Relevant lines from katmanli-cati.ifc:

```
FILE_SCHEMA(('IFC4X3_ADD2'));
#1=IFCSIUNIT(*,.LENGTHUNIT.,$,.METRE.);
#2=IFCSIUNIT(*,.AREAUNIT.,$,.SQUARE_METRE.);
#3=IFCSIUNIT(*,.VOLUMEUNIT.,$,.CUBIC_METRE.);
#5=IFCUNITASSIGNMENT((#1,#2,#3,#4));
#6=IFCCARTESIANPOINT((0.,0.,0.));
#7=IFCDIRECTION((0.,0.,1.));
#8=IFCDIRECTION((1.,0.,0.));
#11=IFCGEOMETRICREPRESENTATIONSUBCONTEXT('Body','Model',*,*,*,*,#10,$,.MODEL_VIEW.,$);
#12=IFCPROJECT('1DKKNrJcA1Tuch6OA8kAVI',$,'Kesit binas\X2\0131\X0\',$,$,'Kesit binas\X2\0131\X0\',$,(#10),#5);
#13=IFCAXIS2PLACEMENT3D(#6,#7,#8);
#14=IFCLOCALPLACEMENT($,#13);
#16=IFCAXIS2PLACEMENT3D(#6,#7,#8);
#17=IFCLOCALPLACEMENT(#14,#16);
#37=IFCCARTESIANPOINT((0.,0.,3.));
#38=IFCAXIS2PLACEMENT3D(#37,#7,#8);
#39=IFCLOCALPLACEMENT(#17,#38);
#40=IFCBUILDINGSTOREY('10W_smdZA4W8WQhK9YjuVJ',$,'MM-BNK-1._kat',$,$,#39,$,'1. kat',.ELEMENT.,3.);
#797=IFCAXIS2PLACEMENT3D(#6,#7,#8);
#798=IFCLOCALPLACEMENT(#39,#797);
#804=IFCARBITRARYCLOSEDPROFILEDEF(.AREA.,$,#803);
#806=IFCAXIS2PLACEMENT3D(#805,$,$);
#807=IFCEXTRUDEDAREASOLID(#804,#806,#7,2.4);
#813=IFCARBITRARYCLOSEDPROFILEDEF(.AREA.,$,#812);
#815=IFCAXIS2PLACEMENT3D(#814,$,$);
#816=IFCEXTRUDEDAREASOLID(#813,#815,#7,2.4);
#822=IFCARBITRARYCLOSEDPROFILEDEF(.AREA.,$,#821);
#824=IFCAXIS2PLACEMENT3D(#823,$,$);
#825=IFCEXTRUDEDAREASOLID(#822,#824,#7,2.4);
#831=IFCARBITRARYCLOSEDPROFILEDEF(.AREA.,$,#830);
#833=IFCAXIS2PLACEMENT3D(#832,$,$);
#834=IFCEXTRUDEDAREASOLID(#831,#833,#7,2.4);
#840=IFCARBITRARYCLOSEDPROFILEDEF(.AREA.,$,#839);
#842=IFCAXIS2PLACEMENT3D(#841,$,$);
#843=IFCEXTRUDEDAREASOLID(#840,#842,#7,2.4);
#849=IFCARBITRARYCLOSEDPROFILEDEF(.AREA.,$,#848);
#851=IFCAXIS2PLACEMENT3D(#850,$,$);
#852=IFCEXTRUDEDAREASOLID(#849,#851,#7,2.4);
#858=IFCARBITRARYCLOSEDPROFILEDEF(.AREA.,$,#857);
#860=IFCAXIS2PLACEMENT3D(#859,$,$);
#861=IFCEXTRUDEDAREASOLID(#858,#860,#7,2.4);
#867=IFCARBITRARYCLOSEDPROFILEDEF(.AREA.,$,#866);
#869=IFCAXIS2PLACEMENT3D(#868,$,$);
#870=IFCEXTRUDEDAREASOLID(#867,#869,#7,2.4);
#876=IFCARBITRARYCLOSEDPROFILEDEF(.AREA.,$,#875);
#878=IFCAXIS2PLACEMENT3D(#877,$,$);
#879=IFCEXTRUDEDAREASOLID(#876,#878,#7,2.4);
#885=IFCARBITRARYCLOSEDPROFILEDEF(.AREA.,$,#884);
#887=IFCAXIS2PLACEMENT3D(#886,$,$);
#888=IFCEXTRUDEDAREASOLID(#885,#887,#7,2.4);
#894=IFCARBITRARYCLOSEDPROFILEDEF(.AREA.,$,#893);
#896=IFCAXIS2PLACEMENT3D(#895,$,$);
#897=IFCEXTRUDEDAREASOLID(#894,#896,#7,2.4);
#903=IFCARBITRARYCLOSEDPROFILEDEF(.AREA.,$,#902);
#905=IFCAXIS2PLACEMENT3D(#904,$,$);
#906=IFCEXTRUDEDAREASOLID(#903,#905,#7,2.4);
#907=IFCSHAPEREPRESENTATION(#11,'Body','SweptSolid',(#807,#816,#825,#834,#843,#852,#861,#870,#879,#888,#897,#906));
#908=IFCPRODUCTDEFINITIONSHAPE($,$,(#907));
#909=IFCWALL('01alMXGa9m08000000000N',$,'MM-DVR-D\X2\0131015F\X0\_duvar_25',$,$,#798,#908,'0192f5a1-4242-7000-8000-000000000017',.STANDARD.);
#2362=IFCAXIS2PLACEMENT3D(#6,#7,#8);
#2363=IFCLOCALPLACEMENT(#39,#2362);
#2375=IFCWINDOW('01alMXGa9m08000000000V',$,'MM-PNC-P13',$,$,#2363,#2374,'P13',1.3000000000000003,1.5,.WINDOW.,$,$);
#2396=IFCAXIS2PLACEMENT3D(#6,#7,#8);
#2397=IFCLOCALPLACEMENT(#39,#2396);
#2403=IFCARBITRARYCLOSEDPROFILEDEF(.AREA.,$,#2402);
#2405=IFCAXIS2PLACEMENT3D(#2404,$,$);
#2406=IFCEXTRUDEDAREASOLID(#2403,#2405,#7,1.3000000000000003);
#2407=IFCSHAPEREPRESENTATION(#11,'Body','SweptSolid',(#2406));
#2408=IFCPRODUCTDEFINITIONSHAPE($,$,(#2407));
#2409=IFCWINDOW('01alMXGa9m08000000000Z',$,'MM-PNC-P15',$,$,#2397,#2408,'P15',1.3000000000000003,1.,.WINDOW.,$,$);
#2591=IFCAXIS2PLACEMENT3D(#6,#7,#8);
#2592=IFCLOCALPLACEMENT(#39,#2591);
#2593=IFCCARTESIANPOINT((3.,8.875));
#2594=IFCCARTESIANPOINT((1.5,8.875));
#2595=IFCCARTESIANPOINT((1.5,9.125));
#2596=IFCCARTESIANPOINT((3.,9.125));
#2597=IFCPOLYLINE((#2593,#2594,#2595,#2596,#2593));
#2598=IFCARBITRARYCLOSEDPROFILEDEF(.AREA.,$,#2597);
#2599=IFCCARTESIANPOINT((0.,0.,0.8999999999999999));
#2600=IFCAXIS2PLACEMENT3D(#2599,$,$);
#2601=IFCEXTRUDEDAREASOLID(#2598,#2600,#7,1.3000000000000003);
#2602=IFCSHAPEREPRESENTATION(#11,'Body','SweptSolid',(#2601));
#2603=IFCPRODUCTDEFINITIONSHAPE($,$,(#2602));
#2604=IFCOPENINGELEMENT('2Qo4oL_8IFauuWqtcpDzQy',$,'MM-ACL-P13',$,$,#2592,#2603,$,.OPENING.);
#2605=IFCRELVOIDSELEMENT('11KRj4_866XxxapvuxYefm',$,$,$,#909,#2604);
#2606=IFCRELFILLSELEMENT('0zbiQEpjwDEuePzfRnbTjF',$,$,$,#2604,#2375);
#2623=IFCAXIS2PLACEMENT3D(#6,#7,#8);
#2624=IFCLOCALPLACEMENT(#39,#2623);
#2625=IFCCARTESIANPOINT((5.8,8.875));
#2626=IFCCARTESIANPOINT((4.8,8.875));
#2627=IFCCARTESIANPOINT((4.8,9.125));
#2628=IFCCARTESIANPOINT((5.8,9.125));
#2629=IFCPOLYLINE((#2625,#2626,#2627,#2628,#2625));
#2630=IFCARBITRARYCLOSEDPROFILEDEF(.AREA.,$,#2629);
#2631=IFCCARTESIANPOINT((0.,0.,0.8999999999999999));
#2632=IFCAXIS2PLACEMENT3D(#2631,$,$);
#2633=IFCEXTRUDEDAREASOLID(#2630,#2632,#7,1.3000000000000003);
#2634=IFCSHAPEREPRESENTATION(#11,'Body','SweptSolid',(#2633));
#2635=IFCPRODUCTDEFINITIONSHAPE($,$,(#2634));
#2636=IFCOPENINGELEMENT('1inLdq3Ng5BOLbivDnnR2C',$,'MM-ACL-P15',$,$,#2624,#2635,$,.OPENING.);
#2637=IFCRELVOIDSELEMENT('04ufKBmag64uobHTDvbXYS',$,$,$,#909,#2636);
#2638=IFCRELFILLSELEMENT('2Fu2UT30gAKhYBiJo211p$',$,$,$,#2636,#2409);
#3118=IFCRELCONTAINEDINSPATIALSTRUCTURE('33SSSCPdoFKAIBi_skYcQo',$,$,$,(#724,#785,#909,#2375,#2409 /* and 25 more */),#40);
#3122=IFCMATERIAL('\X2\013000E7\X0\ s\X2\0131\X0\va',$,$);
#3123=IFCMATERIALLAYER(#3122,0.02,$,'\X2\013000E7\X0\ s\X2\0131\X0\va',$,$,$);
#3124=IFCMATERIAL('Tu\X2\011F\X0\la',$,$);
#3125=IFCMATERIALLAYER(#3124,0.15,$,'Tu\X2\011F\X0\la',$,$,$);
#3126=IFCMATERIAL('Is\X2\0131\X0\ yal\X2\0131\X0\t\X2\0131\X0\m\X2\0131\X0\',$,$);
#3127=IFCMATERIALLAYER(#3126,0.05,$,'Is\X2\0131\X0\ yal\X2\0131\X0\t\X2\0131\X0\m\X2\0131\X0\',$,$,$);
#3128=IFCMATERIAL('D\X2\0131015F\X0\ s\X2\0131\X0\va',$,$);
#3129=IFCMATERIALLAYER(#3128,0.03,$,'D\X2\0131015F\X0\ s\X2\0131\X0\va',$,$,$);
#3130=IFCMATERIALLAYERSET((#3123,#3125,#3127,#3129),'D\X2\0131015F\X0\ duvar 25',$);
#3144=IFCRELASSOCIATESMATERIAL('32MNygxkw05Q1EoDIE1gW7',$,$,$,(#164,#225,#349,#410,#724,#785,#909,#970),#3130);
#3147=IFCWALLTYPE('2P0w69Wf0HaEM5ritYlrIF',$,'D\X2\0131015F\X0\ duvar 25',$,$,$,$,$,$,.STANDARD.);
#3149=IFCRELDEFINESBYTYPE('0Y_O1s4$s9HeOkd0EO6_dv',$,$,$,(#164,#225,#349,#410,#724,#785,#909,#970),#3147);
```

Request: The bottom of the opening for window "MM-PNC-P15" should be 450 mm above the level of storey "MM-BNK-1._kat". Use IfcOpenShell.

```python
import numpy as np
import ifcopenshell
import ifcopenshell.api.geometry
import ifcopenshell.geom
import ifcopenshell.util.element
import ifcopenshell.util.placement
import ifcopenshell.util.shape
import ifcopenshell.util.unit

model = ifcopenshell.open("katmanli-cati.ifc")
unit_scale = ifcopenshell.util.unit.calculate_unit_scale(model)

window = model.by_id(2409)
opening = window.FillsVoids[0].RelatingOpeningElement
storey = ifcopenshell.util.element.get_container(window, ifc_class="IfcBuildingStorey")
level = ifcopenshell.util.placement.get_local_placement(storey.ObjectPlacement)[2, 3]

# The opening's origin need not be at the sill, so measure its lowest point.
shape = ifcopenshell.geom.create_shape(ifcopenshell.geom.settings(), opening)
bottom = ifcopenshell.util.shape.get_shape_bottom_elevation(shape, shape.geometry) / unit_scale
dz = level + 0.45 / unit_scale - bottom

shift = np.array([0.0, 0.0, dz])
# The window is not placed relative to its opening, so move both.
for product in (opening, window):
    matrix = ifcopenshell.util.placement.get_local_placement(product.ObjectPlacement)
    matrix[:3, 3] += shift
    ifcopenshell.api.geometry.edit_object_placement(model, product=product, matrix=matrix, is_si=False)

print(f"moved by {dz * unit_scale:+.3f} m")

model.write("katmanli-cati_edited.ifc")
```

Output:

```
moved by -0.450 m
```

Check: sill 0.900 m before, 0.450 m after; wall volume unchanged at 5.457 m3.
